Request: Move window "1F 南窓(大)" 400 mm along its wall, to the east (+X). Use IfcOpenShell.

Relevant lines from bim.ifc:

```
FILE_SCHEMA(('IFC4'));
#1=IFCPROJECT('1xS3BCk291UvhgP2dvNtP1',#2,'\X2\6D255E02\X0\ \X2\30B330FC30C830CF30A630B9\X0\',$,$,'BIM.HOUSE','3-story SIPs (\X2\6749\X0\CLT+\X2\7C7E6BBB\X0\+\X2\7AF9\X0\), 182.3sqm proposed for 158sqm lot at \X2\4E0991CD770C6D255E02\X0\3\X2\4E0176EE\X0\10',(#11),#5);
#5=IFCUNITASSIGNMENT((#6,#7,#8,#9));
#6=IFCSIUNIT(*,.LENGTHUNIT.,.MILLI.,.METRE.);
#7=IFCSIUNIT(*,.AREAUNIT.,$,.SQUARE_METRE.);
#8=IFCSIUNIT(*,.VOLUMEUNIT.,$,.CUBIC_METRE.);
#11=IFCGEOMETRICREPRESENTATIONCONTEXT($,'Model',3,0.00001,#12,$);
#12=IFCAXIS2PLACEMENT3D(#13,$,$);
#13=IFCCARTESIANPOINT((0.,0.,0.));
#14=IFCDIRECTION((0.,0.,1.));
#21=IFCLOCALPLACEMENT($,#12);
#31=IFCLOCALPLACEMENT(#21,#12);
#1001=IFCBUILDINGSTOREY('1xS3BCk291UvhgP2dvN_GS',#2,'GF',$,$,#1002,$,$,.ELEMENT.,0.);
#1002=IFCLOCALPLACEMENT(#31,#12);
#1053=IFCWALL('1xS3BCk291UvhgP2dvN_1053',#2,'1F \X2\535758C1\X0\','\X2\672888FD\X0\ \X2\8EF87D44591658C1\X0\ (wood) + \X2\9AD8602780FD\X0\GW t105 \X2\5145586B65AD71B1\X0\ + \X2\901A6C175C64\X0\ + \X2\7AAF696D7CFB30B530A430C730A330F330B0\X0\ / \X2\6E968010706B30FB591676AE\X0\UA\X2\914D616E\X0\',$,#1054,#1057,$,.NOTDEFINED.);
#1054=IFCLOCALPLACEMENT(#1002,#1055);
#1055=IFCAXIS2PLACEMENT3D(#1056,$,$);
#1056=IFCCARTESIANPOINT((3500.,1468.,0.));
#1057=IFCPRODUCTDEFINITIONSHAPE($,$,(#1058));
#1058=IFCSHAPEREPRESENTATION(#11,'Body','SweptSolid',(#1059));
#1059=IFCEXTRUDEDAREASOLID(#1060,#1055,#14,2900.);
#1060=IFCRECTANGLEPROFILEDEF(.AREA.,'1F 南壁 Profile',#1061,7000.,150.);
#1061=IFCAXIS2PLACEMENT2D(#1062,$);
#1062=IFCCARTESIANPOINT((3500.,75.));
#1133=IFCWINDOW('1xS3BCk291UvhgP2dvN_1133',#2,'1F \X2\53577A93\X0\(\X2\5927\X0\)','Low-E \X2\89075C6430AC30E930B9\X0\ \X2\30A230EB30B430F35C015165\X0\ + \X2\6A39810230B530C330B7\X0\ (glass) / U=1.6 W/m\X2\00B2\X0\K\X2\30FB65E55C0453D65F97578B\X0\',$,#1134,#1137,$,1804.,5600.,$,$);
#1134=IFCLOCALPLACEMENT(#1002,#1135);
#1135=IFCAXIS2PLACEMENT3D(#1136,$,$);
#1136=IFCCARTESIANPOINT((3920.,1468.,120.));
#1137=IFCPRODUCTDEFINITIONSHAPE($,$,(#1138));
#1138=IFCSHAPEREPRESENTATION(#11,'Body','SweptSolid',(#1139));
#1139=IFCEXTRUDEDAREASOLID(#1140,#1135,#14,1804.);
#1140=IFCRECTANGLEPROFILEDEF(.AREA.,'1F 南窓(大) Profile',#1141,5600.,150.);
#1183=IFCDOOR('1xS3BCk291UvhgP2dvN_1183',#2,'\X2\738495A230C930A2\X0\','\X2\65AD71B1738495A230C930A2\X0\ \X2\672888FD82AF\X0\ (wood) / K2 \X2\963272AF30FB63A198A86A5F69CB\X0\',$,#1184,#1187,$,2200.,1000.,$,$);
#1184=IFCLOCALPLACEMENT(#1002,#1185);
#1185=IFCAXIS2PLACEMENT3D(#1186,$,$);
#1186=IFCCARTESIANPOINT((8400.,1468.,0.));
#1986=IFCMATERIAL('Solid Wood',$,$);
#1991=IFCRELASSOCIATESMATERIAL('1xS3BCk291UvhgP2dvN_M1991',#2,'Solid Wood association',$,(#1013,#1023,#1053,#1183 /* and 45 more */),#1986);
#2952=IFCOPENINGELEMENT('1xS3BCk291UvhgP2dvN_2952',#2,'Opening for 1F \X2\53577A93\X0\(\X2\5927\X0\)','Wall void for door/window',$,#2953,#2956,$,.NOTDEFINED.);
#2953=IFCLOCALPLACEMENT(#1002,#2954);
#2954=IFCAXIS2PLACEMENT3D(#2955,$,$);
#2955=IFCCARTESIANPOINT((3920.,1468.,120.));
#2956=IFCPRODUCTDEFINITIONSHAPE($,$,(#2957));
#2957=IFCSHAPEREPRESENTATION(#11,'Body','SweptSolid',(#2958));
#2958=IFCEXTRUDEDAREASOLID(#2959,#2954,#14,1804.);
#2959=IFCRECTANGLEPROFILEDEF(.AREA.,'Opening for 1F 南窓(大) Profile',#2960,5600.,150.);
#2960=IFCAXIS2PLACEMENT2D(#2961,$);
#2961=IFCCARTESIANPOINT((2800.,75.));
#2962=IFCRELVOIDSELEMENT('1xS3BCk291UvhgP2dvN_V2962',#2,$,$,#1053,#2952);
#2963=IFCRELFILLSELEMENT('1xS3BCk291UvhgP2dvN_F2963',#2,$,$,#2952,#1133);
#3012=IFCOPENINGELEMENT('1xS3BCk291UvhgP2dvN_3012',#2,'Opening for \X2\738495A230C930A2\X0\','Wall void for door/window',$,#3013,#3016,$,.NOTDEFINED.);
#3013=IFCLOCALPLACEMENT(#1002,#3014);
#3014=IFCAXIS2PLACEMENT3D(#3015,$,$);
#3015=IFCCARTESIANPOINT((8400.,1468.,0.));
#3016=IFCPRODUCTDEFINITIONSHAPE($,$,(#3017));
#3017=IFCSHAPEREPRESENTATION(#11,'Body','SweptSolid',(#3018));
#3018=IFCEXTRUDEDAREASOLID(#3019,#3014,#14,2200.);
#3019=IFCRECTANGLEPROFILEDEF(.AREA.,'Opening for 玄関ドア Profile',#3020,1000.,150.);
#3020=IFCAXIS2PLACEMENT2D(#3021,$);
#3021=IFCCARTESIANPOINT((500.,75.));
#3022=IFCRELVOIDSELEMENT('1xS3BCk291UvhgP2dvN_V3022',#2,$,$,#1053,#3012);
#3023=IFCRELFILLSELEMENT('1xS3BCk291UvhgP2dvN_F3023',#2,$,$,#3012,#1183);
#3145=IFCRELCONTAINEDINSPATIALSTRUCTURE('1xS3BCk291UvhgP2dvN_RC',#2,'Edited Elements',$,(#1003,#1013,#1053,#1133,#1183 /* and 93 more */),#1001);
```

```python
import ifcopenshell
import ifcopenshell.api.geometry
import ifcopenshell.util.placement

model = ifcopenshell.open("bim.ifc")

window = model.by_id(1133)
opening = window.FillsVoids[0].RelatingOpeningElement
wall = opening.VoidsElements[0].RelatingBuildingElement

wall_matrix = ifcopenshell.util.placement.get_local_placement(wall.ObjectPlacement)
shift = wall_matrix[:3, 0] * 400.0
before = ifcopenshell.util.placement.get_local_placement(window.ObjectPlacement)[:3, 3].copy()

# The window is not placed relative to its opening, so move both.
for product in (opening, window):
    matrix = ifcopenshell.util.placement.get_local_placement(product.ObjectPlacement)
    matrix[:3, 3] += shift
    ifcopenshell.api.geometry.edit_object_placement(model, product=product, matrix=matrix, is_si=False)

after = ifcopenshell.util.placement.get_local_placement(window.ObjectPlacement)[:3, 3]
print("window moved by", (after - before).round(3) + 0.0)

model.write("bim_rev.ifc")
```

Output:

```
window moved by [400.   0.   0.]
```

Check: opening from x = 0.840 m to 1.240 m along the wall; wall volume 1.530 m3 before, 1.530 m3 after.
